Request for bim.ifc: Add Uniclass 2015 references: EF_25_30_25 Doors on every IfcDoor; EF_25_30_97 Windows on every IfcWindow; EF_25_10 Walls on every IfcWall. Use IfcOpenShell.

First a look at what the model holds.

```python
import ifcopenshell

model = ifcopenshell.open("bim.ifc")
print(model.schema)
print("classifications:", [c.Name for c in model.by_type("IfcClassification")])
for ifc_class in ("IfcDoor", "IfcRoof", "IfcStair", "IfcWall", "IfcWindow"):
    print(ifc_class, len(model.by_type(ifc_class)))
```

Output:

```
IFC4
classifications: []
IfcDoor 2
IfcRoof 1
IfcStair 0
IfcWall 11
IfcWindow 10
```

```python
import ifcopenshell
import ifcopenshell.api.classification

model = ifcopenshell.open("bim.ifc")

system = ifcopenshell.api.classification.add_classification(model, classification="Uniclass 2015")

codes = {
    "IfcDoor": ("EF_25_30_25", "Doors"),
    "IfcWindow": ("EF_25_30_97", "Windows"),
    "IfcWall": ("EF_25_10", "Walls"),
}
for ifc_class, (code, name) in codes.items():
    products = model.by_type(ifc_class)
    ifcopenshell.api.classification.add_reference(
        model, products=products, classification=system, identification=code, name=name
    )
    print(code, len(products))

model.write("bim_v2.ifc")
```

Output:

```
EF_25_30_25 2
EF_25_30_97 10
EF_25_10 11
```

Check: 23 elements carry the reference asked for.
